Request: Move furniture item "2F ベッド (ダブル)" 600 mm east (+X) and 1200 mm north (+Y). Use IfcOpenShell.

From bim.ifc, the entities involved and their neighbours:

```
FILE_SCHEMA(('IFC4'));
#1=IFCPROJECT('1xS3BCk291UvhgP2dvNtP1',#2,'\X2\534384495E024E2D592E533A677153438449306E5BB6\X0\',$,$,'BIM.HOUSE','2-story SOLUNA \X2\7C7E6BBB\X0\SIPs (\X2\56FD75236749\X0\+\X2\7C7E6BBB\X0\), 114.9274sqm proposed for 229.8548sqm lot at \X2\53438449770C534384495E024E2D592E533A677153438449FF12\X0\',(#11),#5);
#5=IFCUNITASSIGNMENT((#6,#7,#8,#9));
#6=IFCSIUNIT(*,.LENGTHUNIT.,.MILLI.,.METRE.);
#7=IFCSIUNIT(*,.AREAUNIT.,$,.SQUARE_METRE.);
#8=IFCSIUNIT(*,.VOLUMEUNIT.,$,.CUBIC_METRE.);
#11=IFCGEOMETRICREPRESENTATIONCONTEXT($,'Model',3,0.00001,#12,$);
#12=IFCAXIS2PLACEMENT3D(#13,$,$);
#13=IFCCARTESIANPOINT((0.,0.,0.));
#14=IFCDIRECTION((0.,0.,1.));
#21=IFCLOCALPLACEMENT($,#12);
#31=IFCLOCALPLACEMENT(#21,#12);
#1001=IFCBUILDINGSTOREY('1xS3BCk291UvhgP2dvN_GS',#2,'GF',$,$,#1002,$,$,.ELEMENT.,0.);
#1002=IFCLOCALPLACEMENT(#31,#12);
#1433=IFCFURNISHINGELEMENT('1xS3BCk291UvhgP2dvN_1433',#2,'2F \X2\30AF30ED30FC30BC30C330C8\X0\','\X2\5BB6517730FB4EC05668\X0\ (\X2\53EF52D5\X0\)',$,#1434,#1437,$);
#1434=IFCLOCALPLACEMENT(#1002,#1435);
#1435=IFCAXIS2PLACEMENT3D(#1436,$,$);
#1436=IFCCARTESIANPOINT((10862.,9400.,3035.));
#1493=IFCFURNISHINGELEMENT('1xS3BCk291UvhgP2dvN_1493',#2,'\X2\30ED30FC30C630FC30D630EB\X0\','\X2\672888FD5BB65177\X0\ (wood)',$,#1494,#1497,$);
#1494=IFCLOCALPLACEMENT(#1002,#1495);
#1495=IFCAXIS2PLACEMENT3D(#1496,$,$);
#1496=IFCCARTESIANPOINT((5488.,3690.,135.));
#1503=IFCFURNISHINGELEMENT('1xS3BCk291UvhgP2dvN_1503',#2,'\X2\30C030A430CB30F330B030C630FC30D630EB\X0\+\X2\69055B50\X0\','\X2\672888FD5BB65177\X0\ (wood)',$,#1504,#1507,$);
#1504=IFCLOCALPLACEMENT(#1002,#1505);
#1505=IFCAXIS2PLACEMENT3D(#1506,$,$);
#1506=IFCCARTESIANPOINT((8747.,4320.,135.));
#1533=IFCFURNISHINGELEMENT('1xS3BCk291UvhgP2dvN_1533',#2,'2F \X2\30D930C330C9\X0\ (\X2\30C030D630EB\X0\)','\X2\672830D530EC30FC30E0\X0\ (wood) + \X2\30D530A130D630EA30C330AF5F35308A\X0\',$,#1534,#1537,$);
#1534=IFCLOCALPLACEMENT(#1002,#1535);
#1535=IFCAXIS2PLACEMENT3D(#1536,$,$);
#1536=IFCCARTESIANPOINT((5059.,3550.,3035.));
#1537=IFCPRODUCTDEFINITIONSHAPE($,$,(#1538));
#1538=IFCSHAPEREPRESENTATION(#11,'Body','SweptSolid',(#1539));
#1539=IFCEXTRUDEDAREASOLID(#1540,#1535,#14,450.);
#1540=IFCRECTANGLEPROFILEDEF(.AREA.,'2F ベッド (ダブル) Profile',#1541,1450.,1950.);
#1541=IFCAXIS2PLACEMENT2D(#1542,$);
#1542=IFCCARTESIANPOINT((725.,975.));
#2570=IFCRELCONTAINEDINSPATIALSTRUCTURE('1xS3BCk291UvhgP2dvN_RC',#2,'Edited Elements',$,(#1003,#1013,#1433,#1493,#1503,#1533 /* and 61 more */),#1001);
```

```python
import ifcopenshell
import ifcopenshell.api.geometry
import ifcopenshell.util.placement

model = ifcopenshell.open("bim.ifc")

item = model.by_id(1533)
matrix = ifcopenshell.util.placement.get_local_placement(item.ObjectPlacement)
matrix[0, 3] += 600.0
matrix[1, 3] += 1200.0
ifcopenshell.api.geometry.edit_object_placement(model, product=item, matrix=matrix, is_si=False)

print(ifcopenshell.util.placement.get_local_placement(item.ObjectPlacement).round(3) + 0.0)

model.write("bim_edited.ifc")
```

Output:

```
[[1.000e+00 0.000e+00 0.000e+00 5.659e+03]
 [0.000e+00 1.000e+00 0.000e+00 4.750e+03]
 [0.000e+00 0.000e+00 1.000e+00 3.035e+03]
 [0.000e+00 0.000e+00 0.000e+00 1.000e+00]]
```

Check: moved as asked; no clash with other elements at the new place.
